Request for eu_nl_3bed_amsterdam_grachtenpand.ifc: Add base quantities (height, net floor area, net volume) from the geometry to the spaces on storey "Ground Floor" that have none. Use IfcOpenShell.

First a look at what the model holds.

```python
import ifcopenshell
import ifcopenshell.util.element
import ifcopenshell.util.unit

model = ifcopenshell.open("eu_nl_3bed_amsterdam_grachtenpand.ifc")
print(model.schema)
for unit_type in ("LENGTHUNIT", "AREAUNIT", "VOLUMEUNIT"):
    print(unit_type, ifcopenshell.util.unit.calculate_unit_scale(model, unit_type))
storey = next(s for s in model.by_type("IfcBuildingStorey") if s.Name == "Ground Floor")
spaces = [e for e in ifcopenshell.util.element.get_decomposition(storey) if e.is_a("IfcSpace")]
for e in sorted(spaces, key=lambda e: e.id()):
    print(e.id(), e.is_a(), e.Name, list(ifcopenshell.util.element.get_psets(e, qtos_only=True)), sep=" | ")
```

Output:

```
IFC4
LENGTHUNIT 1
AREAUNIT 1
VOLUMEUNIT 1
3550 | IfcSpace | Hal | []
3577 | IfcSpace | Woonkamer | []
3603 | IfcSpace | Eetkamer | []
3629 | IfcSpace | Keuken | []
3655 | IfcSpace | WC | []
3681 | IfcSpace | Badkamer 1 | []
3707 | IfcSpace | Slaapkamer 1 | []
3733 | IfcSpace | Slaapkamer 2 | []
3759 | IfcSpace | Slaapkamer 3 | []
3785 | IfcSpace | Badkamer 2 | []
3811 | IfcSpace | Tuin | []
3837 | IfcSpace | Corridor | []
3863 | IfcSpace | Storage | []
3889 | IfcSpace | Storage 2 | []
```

```python
import ifcopenshell
import ifcopenshell.api.pset
import ifcopenshell.geom
import ifcopenshell.util.element
import ifcopenshell.util.shape
import ifcopenshell.util.unit

model = ifcopenshell.open("eu_nl_3bed_amsterdam_grachtenpand.ifc")
unit_scale = ifcopenshell.util.unit.calculate_unit_scale(model)
area_scale = ifcopenshell.util.unit.calculate_unit_scale(model, "AREAUNIT")
volume_scale = ifcopenshell.util.unit.calculate_unit_scale(model, "VOLUMEUNIT")
settings = ifcopenshell.geom.settings()

storey = next(s for s in model.by_type("IfcBuildingStorey") if s.Name == "Ground Floor")
spaces = [e for e in ifcopenshell.util.element.get_decomposition(storey) if e.is_a("IfcSpace")]

for e in sorted(spaces, key=lambda e: e.id()):
    if ifcopenshell.util.element.get_psets(e, qtos_only=True, should_inherit=False):
        continue
    # Geometry comes back in metres, in the element's own axes.
    shape = ifcopenshell.geom.create_shape(settings, e)
    values = {
        "Height": ifcopenshell.util.shape.get_z(shape.geometry) / unit_scale,
        "NetFloorArea": ifcopenshell.util.shape.get_footprint_area(shape.geometry) / area_scale,
        "NetVolume": ifcopenshell.util.shape.get_volume(shape.geometry) / volume_scale,
    }
    qto = ifcopenshell.api.pset.add_qto(model, product=e, name="Qto_SpaceBaseQuantities")
    ifcopenshell.api.pset.edit_qto(model, qto=qto, properties=values)
    print(e.id(), {k: round(v, 3) for k, v in values.items()})

model.write("eu_nl_3bed_amsterdam_grachtenpand_rev.ifc")
```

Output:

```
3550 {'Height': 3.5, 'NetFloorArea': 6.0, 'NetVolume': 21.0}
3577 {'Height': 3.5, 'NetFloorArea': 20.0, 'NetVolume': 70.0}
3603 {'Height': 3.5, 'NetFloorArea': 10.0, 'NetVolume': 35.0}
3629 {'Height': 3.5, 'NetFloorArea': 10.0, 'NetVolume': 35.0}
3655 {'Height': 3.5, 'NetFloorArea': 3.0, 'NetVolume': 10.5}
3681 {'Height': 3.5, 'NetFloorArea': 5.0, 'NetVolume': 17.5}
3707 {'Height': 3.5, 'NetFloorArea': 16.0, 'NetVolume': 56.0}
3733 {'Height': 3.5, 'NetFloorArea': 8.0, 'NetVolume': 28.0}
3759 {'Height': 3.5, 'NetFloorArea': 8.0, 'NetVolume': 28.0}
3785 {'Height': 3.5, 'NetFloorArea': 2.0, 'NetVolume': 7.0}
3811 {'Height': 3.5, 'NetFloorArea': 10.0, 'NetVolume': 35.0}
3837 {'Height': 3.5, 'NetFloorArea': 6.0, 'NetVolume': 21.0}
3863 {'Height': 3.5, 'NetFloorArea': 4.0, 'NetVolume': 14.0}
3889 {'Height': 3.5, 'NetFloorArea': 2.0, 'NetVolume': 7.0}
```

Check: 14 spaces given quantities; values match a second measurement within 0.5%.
